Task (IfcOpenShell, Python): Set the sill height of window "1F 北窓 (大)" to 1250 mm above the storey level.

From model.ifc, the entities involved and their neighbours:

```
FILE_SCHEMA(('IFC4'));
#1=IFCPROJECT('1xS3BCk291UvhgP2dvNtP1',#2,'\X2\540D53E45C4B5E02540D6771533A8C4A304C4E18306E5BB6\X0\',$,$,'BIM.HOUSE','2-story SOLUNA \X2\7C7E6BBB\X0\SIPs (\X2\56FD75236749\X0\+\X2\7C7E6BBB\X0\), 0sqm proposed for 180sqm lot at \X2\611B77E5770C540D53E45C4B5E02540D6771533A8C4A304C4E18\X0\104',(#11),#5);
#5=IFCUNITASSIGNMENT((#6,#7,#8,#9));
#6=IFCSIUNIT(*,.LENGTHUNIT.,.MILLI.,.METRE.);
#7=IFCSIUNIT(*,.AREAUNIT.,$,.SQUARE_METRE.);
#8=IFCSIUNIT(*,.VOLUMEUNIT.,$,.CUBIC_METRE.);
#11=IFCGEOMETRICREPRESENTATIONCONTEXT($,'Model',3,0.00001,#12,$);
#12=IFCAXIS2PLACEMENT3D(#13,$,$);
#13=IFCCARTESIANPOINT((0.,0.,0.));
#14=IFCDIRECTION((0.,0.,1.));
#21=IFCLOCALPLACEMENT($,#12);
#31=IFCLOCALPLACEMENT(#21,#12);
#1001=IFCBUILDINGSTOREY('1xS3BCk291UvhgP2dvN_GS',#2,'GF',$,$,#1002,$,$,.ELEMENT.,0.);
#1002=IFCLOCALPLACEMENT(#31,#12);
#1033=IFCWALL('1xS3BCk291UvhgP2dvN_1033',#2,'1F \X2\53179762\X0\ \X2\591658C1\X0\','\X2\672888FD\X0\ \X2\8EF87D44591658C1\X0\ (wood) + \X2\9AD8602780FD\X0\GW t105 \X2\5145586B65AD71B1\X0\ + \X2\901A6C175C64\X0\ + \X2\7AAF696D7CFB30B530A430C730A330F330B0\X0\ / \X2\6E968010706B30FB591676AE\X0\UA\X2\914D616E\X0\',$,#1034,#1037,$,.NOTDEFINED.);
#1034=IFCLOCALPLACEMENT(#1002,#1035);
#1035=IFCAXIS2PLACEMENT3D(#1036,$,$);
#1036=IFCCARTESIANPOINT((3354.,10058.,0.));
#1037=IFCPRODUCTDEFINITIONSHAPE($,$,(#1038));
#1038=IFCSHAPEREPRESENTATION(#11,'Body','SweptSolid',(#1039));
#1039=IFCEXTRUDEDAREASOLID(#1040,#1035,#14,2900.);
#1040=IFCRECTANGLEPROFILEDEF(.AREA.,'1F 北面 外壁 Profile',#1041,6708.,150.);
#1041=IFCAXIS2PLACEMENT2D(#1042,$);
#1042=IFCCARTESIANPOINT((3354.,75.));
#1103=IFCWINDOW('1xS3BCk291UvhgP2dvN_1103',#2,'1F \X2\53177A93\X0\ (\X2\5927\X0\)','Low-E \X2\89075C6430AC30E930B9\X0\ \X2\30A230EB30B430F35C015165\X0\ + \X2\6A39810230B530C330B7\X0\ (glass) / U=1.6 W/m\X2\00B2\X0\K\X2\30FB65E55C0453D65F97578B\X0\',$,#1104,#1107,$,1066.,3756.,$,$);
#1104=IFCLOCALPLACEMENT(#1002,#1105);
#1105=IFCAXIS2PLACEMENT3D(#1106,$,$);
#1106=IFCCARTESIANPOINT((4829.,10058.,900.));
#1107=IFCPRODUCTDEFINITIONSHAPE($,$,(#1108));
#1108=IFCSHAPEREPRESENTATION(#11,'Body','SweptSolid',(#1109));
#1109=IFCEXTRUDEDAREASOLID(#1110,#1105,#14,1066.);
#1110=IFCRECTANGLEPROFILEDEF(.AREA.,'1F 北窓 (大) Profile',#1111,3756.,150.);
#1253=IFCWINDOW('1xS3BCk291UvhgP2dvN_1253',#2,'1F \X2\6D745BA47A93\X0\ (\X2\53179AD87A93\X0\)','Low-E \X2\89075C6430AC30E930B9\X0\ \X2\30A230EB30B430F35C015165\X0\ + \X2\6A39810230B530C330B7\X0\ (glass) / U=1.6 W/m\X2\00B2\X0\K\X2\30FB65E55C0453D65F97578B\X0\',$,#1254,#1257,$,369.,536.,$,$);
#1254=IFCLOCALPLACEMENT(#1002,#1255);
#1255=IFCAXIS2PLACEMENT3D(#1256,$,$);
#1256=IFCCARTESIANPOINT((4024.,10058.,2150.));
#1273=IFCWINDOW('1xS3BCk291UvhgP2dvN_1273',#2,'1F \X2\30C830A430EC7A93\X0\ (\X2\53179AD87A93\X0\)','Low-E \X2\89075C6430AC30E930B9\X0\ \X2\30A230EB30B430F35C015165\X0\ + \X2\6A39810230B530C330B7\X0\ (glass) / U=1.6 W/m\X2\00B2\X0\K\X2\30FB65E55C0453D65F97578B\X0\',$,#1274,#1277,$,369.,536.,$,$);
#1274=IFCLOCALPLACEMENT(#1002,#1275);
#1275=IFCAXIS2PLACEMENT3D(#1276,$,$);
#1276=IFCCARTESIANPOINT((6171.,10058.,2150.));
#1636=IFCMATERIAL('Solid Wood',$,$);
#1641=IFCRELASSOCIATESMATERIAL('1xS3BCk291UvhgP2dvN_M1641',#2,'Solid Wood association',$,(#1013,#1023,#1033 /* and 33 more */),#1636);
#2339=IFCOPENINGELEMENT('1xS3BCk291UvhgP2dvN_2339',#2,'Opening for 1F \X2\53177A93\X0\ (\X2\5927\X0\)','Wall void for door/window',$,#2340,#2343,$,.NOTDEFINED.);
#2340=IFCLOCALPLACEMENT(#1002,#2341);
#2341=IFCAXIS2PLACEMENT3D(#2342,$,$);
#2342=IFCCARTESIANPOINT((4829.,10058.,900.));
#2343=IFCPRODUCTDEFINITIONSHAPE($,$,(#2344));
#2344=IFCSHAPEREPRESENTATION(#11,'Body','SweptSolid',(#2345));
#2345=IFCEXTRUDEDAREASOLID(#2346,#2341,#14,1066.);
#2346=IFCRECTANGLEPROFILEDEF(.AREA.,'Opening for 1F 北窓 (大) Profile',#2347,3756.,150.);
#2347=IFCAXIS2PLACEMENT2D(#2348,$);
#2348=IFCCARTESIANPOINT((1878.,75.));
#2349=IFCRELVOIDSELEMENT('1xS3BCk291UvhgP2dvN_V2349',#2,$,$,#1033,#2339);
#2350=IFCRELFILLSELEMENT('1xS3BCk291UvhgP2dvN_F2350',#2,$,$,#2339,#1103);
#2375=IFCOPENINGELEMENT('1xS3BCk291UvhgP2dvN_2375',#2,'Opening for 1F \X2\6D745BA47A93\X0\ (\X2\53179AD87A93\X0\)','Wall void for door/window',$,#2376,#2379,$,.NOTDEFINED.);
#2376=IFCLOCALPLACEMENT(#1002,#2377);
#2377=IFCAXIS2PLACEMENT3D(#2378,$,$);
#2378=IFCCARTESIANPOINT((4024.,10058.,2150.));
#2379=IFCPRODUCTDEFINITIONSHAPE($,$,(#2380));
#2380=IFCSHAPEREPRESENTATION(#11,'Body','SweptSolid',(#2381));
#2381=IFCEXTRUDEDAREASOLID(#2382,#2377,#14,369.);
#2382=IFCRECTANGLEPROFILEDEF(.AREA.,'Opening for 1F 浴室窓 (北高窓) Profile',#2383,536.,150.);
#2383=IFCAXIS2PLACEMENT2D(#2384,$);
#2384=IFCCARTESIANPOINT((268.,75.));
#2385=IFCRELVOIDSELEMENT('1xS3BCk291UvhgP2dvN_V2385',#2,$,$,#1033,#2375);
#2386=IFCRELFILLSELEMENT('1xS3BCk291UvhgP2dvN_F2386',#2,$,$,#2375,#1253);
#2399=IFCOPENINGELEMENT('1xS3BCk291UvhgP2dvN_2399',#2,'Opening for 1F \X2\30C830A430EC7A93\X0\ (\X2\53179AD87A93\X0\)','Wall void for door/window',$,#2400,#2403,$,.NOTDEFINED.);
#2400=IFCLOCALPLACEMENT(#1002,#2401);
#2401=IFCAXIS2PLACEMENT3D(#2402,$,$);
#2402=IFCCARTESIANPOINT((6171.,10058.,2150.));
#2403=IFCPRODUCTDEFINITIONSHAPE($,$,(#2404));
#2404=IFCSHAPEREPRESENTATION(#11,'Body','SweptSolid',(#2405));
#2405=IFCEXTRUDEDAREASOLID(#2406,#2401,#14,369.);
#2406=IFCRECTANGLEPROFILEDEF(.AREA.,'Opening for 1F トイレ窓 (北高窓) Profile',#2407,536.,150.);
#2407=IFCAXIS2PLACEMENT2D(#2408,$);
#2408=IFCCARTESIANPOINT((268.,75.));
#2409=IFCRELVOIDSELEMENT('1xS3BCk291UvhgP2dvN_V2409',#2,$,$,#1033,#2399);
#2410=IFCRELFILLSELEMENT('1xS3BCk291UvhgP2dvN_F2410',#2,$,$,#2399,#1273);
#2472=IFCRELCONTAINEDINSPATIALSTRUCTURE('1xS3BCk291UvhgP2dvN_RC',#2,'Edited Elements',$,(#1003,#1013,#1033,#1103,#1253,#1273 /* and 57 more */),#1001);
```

```python
import numpy as np
import ifcopenshell
import ifcopenshell.api.geometry
import ifcopenshell.geom
import ifcopenshell.util.element
import ifcopenshell.util.placement
import ifcopenshell.util.shape
import ifcopenshell.util.unit

model = ifcopenshell.open("model.ifc")
unit_scale = ifcopenshell.util.unit.calculate_unit_scale(model)

window = model.by_guid("1xS3BCk291UvhgP2dvN_1103")
opening = window.FillsVoids[0].RelatingOpeningElement
storey = ifcopenshell.util.element.get_container(window, ifc_class="IfcBuildingStorey")
level = ifcopenshell.util.placement.get_local_placement(storey.ObjectPlacement)[2, 3]

# The opening's origin need not be at the sill, so measure its lowest point.
shape = ifcopenshell.geom.create_shape(ifcopenshell.geom.settings(), opening)
bottom = ifcopenshell.util.shape.get_shape_bottom_elevation(shape, shape.geometry) / unit_scale
dz = level + 1250.0 - bottom

shift = np.array([0.0, 0.0, dz])
# The window is not placed relative to its opening, so move both.
for product in (opening, window):
    matrix = ifcopenshell.util.placement.get_local_placement(product.ObjectPlacement)
    matrix[:3, 3] += shift
    ifcopenshell.api.geometry.edit_object_placement(model, product=product, matrix=matrix, is_si=False)

print(f"moved by {dz * unit_scale:+.3f} m")

model.write("model_edited.ifc")
```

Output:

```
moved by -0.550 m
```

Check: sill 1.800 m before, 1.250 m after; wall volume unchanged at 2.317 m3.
